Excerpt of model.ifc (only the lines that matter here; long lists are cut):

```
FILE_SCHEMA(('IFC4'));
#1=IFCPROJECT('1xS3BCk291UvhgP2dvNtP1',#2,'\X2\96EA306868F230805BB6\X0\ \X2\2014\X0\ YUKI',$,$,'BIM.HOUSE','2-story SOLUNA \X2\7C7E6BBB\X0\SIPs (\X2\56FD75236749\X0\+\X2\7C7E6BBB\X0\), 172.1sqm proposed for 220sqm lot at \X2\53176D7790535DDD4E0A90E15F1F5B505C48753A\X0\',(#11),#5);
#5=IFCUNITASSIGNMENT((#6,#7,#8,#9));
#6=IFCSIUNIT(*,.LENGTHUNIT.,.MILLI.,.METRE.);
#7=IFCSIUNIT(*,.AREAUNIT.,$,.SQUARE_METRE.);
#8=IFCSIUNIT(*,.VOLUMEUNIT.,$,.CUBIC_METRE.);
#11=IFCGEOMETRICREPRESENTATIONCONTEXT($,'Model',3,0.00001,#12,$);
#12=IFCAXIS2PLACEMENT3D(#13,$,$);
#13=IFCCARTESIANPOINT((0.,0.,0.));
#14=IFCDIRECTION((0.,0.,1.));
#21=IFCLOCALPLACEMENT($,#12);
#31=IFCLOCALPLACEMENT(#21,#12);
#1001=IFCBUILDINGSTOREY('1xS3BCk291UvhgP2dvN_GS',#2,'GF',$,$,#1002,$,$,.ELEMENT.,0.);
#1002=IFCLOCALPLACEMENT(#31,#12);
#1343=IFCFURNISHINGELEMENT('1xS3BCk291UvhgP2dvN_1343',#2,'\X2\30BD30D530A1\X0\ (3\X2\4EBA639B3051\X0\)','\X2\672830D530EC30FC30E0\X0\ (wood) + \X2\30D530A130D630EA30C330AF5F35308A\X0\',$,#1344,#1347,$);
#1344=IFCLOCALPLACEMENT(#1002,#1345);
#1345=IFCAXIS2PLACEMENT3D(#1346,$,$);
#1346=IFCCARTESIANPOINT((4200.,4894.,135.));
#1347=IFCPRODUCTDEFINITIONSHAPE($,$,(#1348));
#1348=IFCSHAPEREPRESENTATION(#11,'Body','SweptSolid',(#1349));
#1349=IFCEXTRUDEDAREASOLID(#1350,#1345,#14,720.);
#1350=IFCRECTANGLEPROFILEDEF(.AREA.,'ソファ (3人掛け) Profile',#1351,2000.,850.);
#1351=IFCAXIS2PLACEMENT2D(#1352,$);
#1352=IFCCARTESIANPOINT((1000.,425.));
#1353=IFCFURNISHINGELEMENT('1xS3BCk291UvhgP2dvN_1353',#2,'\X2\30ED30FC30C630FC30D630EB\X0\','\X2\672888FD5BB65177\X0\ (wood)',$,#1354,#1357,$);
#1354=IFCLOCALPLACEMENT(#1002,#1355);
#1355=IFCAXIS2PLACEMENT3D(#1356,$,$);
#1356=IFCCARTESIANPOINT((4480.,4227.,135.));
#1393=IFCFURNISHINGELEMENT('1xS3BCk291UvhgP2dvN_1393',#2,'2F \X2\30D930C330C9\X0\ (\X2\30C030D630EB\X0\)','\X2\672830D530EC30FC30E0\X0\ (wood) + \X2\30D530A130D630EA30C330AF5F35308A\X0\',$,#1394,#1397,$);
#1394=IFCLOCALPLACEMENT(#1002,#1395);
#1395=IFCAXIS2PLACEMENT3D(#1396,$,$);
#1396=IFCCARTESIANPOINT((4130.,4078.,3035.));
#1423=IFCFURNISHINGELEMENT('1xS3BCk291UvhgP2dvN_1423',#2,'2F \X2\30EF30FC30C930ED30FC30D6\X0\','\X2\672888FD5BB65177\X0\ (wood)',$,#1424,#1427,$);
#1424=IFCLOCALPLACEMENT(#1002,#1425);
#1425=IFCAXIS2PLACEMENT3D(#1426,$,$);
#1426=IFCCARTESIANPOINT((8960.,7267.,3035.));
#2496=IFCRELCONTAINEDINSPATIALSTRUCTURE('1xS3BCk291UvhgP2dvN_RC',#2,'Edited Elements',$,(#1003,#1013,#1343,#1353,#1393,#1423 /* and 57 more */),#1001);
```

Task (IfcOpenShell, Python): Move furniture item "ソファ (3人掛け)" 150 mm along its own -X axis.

```python
import ifcopenshell
import ifcopenshell.api.geometry
import ifcopenshell.util.placement

model = ifcopenshell.open("model.ifc")

item = model.by_guid("1xS3BCk291UvhgP2dvN_1343")
matrix = ifcopenshell.util.placement.get_local_placement(item.ObjectPlacement)
matrix[:3, 3] -= matrix[:3, 0] * 150.0
ifcopenshell.api.geometry.edit_object_placement(model, product=item, matrix=matrix, is_si=False)

print(ifcopenshell.util.placement.get_local_placement(item.ObjectPlacement).round(3) + 0.0)

model.write("model-out.ifc")
```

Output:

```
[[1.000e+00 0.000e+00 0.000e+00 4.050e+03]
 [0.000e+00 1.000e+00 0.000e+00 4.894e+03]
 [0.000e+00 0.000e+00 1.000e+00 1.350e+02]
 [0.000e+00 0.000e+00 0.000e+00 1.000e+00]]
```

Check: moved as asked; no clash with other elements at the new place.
